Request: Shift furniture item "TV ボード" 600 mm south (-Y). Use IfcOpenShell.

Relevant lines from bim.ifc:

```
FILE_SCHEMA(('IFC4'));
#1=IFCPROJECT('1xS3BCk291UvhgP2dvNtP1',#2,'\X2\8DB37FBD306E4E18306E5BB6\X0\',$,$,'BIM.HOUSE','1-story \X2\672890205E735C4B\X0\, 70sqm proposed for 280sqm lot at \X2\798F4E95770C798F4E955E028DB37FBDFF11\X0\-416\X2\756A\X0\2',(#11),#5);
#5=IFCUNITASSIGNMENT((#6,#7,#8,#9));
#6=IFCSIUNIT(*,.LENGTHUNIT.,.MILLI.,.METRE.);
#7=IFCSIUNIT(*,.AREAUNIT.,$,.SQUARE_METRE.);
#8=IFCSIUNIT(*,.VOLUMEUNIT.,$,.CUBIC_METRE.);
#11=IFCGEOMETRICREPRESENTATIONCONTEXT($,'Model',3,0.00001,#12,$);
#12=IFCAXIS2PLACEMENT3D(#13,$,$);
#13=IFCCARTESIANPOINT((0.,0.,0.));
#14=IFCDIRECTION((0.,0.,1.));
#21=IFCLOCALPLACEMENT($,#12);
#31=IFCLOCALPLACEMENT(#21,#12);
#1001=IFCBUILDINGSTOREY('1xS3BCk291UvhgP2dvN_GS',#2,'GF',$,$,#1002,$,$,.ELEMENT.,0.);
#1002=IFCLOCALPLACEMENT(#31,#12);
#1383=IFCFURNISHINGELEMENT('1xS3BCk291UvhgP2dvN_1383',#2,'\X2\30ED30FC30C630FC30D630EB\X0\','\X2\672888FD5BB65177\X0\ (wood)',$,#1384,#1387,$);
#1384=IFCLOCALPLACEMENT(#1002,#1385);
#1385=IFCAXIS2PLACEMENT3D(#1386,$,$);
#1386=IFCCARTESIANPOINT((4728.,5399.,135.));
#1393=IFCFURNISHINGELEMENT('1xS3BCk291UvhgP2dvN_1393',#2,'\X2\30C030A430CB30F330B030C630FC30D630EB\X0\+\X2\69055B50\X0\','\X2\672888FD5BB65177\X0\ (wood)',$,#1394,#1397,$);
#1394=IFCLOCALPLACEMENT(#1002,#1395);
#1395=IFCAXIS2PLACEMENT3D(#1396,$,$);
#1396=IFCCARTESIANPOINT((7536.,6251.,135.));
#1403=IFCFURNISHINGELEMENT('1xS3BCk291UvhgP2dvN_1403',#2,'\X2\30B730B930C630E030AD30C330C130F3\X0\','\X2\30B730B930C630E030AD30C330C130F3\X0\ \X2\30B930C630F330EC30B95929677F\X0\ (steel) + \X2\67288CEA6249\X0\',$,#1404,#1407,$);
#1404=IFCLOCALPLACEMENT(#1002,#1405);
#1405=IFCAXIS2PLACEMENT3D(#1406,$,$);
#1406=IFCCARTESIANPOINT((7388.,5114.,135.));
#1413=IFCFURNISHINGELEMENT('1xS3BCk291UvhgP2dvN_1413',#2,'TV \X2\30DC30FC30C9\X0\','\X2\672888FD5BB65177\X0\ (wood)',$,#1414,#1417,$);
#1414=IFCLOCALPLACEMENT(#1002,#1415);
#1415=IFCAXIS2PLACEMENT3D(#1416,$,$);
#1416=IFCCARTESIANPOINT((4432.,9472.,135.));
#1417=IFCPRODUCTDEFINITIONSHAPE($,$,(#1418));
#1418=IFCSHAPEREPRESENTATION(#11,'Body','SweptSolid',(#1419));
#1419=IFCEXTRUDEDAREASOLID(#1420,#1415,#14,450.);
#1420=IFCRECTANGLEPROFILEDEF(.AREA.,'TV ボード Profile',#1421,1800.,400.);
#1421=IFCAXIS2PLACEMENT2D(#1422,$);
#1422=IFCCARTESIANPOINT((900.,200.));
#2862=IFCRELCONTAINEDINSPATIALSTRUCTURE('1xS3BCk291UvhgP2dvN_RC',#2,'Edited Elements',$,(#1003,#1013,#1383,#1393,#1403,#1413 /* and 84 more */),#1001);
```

```python
import ifcopenshell
import ifcopenshell.api.geometry
import ifcopenshell.util.placement
import ifcopenshell.util.unit

model = ifcopenshell.open("bim.ifc")
unit_scale = ifcopenshell.util.unit.calculate_unit_scale(model)

item = model.by_id(1413)
matrix = ifcopenshell.util.placement.get_local_placement(item.ObjectPlacement)
matrix[1, 3] -= 0.6 / unit_scale
ifcopenshell.api.geometry.edit_object_placement(model, product=item, matrix=matrix, is_si=False)

print(ifcopenshell.util.placement.get_local_placement(item.ObjectPlacement).round(3) + 0.0)

model.write("bim_rev.ifc")
```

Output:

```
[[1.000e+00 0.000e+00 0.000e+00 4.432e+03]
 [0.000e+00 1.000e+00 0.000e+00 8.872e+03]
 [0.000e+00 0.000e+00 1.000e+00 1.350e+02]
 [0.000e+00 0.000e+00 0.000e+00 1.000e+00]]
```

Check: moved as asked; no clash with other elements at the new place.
